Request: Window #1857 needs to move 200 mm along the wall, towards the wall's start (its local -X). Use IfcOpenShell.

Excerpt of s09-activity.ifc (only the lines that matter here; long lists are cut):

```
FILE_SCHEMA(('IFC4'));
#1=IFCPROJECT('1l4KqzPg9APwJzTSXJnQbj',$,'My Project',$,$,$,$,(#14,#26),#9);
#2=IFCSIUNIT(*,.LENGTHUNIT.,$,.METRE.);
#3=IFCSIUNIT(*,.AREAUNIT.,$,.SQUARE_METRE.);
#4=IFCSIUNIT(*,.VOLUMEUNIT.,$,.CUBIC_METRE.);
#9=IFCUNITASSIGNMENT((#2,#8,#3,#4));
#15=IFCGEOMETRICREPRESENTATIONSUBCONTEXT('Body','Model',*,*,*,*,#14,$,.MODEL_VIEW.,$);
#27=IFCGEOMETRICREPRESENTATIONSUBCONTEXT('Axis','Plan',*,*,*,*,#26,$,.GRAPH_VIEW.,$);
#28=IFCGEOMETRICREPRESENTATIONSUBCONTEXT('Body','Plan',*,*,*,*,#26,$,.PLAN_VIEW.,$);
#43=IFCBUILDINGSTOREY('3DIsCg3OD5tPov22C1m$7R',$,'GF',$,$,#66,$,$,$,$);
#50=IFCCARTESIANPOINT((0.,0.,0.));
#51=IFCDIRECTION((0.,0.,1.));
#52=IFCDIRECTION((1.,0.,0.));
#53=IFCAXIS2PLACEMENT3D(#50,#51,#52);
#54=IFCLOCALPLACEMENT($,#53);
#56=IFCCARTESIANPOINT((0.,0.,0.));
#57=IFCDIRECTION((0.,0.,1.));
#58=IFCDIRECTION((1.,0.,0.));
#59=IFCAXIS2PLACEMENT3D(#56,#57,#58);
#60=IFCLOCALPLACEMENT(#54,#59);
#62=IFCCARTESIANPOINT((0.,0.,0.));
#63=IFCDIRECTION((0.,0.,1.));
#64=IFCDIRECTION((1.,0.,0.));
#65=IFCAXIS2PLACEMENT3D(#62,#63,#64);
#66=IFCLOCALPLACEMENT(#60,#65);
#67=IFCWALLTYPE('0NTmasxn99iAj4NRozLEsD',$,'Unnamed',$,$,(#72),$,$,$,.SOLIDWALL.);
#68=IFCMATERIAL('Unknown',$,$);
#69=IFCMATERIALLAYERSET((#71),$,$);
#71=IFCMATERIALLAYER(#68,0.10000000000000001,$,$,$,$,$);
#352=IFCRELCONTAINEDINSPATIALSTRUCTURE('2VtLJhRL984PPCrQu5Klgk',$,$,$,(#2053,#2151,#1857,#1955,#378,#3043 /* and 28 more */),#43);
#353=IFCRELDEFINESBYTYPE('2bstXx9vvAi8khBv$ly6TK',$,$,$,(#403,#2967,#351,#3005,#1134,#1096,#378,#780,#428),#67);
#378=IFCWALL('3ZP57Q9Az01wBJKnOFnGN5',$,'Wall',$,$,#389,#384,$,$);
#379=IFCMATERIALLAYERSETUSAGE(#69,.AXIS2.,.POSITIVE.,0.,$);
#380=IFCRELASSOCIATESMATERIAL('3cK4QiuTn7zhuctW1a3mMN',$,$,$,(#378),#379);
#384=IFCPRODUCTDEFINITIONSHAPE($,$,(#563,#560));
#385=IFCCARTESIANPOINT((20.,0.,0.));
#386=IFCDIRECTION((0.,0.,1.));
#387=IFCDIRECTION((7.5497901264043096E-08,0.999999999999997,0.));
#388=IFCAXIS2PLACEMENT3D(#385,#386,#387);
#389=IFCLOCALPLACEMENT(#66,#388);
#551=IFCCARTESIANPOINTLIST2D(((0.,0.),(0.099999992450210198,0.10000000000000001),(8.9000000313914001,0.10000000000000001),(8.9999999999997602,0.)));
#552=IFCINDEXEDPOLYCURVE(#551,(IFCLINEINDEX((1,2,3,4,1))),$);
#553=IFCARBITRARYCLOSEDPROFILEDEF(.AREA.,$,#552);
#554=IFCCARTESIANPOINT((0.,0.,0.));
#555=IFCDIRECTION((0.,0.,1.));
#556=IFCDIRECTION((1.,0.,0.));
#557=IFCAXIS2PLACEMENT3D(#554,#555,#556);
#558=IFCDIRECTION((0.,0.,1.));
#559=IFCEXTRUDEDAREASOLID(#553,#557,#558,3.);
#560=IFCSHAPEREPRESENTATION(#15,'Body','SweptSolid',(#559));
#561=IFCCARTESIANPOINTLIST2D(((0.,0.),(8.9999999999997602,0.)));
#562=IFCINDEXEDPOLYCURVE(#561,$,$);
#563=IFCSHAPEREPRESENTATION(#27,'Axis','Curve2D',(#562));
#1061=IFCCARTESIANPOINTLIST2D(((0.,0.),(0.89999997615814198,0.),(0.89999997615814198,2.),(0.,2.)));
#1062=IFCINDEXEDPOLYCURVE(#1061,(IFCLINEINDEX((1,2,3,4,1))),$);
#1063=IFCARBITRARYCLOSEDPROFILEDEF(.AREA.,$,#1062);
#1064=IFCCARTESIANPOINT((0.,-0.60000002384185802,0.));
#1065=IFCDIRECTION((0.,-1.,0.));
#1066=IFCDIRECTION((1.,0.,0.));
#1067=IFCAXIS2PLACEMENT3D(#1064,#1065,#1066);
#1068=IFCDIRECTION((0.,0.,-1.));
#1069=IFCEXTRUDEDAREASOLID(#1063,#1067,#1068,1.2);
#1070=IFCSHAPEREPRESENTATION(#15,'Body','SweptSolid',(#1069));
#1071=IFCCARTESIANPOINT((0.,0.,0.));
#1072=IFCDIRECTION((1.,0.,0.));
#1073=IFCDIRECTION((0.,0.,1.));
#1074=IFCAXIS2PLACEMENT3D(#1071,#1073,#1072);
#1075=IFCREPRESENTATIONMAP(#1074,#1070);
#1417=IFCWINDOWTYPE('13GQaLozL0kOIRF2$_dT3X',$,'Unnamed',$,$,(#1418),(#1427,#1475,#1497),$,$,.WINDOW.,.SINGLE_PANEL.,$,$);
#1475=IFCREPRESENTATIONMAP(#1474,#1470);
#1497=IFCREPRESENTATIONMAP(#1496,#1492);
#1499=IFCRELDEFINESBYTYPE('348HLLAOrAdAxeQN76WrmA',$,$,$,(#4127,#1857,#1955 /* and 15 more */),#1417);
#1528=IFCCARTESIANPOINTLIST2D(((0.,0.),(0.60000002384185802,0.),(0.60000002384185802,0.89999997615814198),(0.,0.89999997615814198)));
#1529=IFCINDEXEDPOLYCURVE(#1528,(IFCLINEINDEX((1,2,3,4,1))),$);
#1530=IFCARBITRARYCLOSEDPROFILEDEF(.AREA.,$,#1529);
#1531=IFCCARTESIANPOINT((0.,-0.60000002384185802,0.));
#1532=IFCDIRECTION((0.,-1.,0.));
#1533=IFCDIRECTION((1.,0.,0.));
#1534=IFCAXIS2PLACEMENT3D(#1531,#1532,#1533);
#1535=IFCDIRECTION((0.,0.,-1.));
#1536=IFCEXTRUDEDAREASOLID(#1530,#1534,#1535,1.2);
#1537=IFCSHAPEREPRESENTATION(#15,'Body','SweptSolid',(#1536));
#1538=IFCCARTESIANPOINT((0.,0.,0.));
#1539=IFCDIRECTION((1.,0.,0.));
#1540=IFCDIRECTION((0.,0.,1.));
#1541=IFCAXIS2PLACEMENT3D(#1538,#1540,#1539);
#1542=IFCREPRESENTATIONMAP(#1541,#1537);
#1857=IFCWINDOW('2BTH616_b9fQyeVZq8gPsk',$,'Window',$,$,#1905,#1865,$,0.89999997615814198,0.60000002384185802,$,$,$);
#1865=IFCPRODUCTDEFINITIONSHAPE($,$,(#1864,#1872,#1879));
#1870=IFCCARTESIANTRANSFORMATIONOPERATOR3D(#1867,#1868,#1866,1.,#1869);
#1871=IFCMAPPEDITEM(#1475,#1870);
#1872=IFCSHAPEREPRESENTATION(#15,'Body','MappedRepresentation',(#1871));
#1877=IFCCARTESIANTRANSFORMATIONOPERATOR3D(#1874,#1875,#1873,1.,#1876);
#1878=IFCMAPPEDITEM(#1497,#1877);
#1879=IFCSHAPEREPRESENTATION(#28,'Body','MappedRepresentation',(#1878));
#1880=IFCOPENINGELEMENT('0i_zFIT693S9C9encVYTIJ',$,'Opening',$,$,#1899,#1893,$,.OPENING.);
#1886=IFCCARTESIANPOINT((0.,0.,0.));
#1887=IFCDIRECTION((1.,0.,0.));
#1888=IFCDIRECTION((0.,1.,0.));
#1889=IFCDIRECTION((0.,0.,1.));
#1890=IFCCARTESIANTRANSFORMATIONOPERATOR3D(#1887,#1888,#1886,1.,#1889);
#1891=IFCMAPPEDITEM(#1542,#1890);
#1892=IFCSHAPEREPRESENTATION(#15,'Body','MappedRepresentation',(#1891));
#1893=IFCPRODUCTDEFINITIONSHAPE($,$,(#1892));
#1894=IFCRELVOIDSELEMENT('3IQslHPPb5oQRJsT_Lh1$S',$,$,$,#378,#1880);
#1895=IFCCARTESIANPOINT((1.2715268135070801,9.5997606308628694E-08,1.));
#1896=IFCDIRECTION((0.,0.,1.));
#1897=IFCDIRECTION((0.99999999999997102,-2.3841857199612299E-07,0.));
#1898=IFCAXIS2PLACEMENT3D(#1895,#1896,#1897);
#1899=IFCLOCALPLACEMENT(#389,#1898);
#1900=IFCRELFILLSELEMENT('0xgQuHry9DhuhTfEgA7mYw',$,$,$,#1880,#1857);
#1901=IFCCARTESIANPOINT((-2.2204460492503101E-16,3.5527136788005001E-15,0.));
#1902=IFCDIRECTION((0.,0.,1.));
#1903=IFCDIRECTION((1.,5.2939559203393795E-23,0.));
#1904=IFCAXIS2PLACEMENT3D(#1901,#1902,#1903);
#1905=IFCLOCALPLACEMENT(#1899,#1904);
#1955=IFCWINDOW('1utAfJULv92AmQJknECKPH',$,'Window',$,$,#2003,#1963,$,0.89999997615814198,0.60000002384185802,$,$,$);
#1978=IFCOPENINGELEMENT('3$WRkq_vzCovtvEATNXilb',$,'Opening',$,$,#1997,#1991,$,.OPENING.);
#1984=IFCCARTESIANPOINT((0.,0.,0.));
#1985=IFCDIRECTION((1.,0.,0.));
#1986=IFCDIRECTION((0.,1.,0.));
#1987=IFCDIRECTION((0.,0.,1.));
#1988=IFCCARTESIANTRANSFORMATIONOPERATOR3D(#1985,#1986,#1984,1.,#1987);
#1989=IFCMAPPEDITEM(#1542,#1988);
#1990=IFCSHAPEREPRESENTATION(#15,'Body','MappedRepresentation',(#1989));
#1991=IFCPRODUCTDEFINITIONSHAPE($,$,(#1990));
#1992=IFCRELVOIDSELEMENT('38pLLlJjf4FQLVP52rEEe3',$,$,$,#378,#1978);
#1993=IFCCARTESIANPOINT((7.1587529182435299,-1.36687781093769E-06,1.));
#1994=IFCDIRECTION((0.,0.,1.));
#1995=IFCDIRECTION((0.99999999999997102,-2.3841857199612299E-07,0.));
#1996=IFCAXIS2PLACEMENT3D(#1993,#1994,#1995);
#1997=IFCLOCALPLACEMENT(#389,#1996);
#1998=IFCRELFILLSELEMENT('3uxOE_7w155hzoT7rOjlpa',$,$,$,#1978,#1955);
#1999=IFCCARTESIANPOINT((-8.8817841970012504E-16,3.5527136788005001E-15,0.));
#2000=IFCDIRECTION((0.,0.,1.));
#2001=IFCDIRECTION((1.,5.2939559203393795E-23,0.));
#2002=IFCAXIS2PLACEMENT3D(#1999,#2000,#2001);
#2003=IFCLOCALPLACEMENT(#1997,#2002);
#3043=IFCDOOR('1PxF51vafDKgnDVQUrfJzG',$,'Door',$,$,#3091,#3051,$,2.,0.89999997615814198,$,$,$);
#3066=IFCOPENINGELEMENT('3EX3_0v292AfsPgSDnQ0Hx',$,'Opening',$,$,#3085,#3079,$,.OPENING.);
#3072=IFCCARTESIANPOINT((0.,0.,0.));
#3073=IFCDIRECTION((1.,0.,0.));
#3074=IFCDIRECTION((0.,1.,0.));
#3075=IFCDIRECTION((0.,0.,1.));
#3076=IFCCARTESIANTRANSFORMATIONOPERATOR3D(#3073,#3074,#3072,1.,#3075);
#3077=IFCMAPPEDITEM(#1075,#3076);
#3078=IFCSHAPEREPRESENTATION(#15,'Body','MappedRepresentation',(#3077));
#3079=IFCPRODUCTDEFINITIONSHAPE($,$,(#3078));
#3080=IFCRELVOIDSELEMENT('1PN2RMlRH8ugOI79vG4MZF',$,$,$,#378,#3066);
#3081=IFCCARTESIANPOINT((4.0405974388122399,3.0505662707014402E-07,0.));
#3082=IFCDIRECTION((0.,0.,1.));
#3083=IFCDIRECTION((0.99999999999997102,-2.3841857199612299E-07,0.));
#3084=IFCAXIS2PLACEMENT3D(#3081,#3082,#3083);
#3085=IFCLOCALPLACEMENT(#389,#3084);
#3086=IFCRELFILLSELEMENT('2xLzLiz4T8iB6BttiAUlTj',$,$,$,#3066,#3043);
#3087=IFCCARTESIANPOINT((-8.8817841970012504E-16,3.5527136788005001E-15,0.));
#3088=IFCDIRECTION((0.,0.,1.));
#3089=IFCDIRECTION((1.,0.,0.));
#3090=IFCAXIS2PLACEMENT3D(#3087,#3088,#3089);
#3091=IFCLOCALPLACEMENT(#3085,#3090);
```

```python
import ifcopenshell
import ifcopenshell.api.geometry
import ifcopenshell.util.placement
import ifcopenshell.util.unit

model = ifcopenshell.open("s09-activity.ifc")
unit_scale = ifcopenshell.util.unit.calculate_unit_scale(model)

window = model.by_guid("2BTH616_b9fQyeVZq8gPsk")
opening = window.FillsVoids[0].RelatingOpeningElement
wall = opening.VoidsElements[0].RelatingBuildingElement

wall_matrix = ifcopenshell.util.placement.get_local_placement(wall.ObjectPlacement)
shift = wall_matrix[:3, 0] * -0.2 / unit_scale
before = ifcopenshell.util.placement.get_local_placement(window.ObjectPlacement)[:3, 3].copy()

# The window is placed relative to its opening, so it follows when the opening moves.
matrix = ifcopenshell.util.placement.get_local_placement(opening.ObjectPlacement)
matrix[:3, 3] += shift
ifcopenshell.api.geometry.edit_object_placement(
    model, product=opening, matrix=matrix, is_si=False, should_transform_children=True
)

after = ifcopenshell.util.placement.get_local_placement(window.ObjectPlacement)[:3, 3]
print("window moved by", (after - before).round(3) + 0.0)

model.write("s09-activity-out.ifc")
```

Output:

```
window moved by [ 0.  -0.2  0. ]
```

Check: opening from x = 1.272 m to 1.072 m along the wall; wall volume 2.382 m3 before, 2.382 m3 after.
